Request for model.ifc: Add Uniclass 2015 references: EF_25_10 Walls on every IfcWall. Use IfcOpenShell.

First a look at what the model holds.

```python
import ifcopenshell

model = ifcopenshell.open("model.ifc")
print(model.schema)
print("classifications:", [c.Name for c in model.by_type("IfcClassification")])
for ifc_class in ("IfcDoor", "IfcRoof", "IfcStair", "IfcWall", "IfcWindow"):
    print(ifc_class, len(model.by_type(ifc_class)))
```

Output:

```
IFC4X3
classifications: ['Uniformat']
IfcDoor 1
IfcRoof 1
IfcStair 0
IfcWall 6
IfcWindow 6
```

```python
import ifcopenshell
import ifcopenshell.api.classification

model = ifcopenshell.open("model.ifc")

system = ifcopenshell.api.classification.add_classification(model, classification="Uniclass 2015")

codes = {
    "IfcWall": ("EF_25_10", "Walls"),
}
for ifc_class, (code, name) in codes.items():
    products = model.by_type(ifc_class)
    ifcopenshell.api.classification.add_reference(
        model, products=products, classification=system, identification=code, name=name
    )
    print(code, len(products))

model.write("model_v2.ifc")
```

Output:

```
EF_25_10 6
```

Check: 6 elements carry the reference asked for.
